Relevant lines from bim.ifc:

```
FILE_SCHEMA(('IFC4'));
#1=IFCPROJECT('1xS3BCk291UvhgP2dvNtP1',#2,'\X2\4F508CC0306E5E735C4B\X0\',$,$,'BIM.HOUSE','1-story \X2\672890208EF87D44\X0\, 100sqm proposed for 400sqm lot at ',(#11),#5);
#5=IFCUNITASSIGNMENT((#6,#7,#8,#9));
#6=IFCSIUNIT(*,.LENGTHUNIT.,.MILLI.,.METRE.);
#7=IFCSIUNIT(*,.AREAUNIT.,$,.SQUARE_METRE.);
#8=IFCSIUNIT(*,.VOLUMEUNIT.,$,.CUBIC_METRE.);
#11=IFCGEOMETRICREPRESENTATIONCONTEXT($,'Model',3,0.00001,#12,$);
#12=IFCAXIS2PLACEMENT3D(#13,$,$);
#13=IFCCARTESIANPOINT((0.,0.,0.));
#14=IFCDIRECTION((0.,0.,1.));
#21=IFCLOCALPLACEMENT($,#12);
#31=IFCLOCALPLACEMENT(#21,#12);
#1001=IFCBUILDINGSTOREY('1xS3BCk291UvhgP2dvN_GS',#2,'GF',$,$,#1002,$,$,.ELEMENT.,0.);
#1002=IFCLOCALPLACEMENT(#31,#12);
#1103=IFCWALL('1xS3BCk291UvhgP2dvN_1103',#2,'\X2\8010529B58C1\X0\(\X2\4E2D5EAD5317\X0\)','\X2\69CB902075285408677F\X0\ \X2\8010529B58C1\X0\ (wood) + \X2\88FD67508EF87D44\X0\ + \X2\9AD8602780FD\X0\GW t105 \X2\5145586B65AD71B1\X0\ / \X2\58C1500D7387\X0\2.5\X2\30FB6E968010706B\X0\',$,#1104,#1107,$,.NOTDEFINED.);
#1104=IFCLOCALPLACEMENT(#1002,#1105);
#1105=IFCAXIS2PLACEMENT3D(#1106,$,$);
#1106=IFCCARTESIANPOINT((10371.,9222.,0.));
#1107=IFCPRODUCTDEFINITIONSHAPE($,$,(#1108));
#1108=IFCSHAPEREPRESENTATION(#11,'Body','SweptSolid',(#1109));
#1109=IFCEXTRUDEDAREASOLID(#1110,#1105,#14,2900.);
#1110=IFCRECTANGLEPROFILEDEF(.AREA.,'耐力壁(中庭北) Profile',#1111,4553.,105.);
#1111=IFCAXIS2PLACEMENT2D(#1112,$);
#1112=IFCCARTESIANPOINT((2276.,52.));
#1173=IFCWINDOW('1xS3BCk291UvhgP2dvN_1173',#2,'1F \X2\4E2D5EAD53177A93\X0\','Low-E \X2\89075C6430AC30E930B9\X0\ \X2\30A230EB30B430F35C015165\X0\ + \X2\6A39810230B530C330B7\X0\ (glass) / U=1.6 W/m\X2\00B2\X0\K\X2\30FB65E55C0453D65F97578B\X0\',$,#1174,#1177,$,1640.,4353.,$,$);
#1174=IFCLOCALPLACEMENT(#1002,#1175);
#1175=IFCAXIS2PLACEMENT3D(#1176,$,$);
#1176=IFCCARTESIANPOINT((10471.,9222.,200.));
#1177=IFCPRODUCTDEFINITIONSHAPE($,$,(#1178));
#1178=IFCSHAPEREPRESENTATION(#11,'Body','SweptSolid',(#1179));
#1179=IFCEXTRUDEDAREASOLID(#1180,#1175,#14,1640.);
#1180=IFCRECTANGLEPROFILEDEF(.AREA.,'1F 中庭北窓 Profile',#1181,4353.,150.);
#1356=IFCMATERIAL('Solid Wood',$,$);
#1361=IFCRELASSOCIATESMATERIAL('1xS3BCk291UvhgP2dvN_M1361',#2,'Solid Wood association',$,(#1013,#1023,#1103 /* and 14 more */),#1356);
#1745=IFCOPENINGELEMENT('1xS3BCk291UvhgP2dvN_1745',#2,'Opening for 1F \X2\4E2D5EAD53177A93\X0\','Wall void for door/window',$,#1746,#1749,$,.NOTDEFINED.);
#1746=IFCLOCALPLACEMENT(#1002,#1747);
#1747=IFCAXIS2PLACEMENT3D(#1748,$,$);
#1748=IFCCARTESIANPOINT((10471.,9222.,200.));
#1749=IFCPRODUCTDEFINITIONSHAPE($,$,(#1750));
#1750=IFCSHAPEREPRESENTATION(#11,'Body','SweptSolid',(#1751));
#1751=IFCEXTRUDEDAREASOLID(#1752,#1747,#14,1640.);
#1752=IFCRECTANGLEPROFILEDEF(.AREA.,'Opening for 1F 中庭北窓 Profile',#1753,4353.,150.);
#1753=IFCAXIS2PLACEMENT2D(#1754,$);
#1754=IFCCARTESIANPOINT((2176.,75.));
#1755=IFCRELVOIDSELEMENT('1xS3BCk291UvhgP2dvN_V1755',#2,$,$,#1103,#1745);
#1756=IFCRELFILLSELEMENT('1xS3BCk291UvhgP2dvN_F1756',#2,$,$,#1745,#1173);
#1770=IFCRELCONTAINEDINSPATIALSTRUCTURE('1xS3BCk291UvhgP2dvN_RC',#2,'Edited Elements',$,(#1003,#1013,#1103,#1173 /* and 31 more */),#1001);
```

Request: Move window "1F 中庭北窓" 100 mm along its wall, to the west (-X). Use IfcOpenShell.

```python
import ifcopenshell
import ifcopenshell.api.geometry
import ifcopenshell.util.placement

model = ifcopenshell.open("bim.ifc")

window = model.by_guid("1xS3BCk291UvhgP2dvN_1173")
opening = window.FillsVoids[0].RelatingOpeningElement
wall = opening.VoidsElements[0].RelatingBuildingElement

wall_matrix = ifcopenshell.util.placement.get_local_placement(wall.ObjectPlacement)
shift = wall_matrix[:3, 0] * -100.0
before = ifcopenshell.util.placement.get_local_placement(window.ObjectPlacement)[:3, 3].copy()

# The window is not placed relative to its opening, so move both.
for product in (opening, window):
    matrix = ifcopenshell.util.placement.get_local_placement(product.ObjectPlacement)
    matrix[:3, 3] += shift
    ifcopenshell.api.geometry.edit_object_placement(model, product=product, matrix=matrix, is_si=False)

after = ifcopenshell.util.placement.get_local_placement(window.ObjectPlacement)[:3, 3]
print("window moved by", (after - before).round(3) + 0.0)

model.write("bim-out.ifc")
```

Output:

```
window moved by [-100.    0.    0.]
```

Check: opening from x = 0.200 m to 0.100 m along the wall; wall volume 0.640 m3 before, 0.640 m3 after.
